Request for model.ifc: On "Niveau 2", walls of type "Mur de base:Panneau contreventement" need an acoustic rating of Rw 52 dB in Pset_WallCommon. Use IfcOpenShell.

First a look at what the model holds.

```python
import ifcopenshell
import ifcopenshell.util.element

model = ifcopenshell.open("model.ifc")
print(model.schema)
storey = next(s for s in model.by_type("IfcBuildingStorey") if s.Name == "Niveau 2")
walls = [e for e in ifcopenshell.util.element.get_decomposition(storey) if e.is_a("IfcWall")]
seen = {}
for e in walls:
    element_type = ifcopenshell.util.element.get_type(e)
    key = (element_type.Name if element_type != e and element_type else None, ifcopenshell.util.element.get_pset(e, "Pset_WallCommon", "AcousticRating"))
    seen[key] = seen.get(key, 0) + 1
for (name, value), count in sorted(seen.items(), key=str):
    print(count, "x", name, "|", value)
```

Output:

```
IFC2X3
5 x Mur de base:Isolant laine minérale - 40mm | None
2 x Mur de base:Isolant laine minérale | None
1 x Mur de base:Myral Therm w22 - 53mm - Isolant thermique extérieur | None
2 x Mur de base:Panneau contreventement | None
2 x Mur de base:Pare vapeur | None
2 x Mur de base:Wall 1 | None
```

```python
import ifcopenshell
import ifcopenshell.api.pset
import ifcopenshell.util.element

model = ifcopenshell.open("model.ifc")

storey = next(s for s in model.by_type("IfcBuildingStorey") if s.Name == "Niveau 2")
walls = [e for e in ifcopenshell.util.element.get_decomposition(storey) if e.is_a("IfcWall")]

count = 0
for e in walls:
    element_type = ifcopenshell.util.element.get_type(e)
    if element_type in (None, e) or element_type.Name != "Mur de base:Panneau contreventement":
        continue
    # add_pset returns the element's existing set when there is one.
    pset = ifcopenshell.api.pset.add_pset(model, product=e, name="Pset_WallCommon")
    ifcopenshell.api.pset.edit_pset(model, pset=pset, properties={"AcousticRating": "Rw 52 dB"})
    count += 1

print(count, "walls updated")

model.write("model_rev.ifc")
```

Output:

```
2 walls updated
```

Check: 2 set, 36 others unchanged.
